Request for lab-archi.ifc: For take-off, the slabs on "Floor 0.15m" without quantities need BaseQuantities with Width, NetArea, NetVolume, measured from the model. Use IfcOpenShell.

First a look at what the model holds.

```python
import ifcopenshell
import ifcopenshell.util.element
import ifcopenshell.util.unit

model = ifcopenshell.open("lab-archi.ifc")
print(model.schema)
for unit_type in ("LENGTHUNIT", "AREAUNIT", "VOLUMEUNIT"):
    print(unit_type, ifcopenshell.util.unit.calculate_unit_scale(model, unit_type))
storey = next(s for s in model.by_type("IfcBuildingStorey") if s.Name == "Floor 0.15m")
slabs = [e for e in ifcopenshell.util.element.get_decomposition(storey) if e.is_a("IfcSlab")]
for e in sorted(slabs, key=lambda e: e.id()):
    print(e.id(), e.is_a(), e.Name, list(ifcopenshell.util.element.get_psets(e, qtos_only=True)), sep=" | ")
```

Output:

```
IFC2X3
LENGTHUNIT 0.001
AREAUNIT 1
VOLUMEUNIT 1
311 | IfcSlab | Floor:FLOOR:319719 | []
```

```python
import ifcopenshell
import ifcopenshell.api.pset
import ifcopenshell.geom
import ifcopenshell.util.element
import ifcopenshell.util.shape
import ifcopenshell.util.unit

model = ifcopenshell.open("lab-archi.ifc")
unit_scale = ifcopenshell.util.unit.calculate_unit_scale(model)
area_scale = ifcopenshell.util.unit.calculate_unit_scale(model, "AREAUNIT")
volume_scale = ifcopenshell.util.unit.calculate_unit_scale(model, "VOLUMEUNIT")
settings = ifcopenshell.geom.settings()

storey = next(s for s in model.by_type("IfcBuildingStorey") if s.Name == "Floor 0.15m")
slabs = [e for e in ifcopenshell.util.element.get_decomposition(storey) if e.is_a("IfcSlab")]

for e in sorted(slabs, key=lambda e: e.id()):
    if ifcopenshell.util.element.get_psets(e, qtos_only=True, should_inherit=False):
        continue
    # Geometry comes back in metres, in the element's own axes.
    shape = ifcopenshell.geom.create_shape(settings, e)
    values = {
        "Width": ifcopenshell.util.shape.get_z(shape.geometry) / unit_scale,
        "NetArea": ifcopenshell.util.shape.get_footprint_area(shape.geometry) / area_scale,
        "NetVolume": ifcopenshell.util.shape.get_volume(shape.geometry) / volume_scale,
    }
    qto = ifcopenshell.api.pset.add_qto(model, product=e, name="BaseQuantities")
    ifcopenshell.api.pset.edit_qto(model, qto=qto, properties=values)
    print(e.id(), {k: round(v, 3) for k, v in values.items()})

model.write("lab-archi_rev.ifc")
```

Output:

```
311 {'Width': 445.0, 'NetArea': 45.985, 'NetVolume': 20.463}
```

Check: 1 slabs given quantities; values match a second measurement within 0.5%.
